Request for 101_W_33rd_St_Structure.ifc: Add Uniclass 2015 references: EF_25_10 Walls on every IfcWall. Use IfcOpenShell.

First a look at what the model holds.

```python
import ifcopenshell

model = ifcopenshell.open("101_W_33rd_St_Structure.ifc")
print(model.schema)
print("classifications:", [c.Name for c in model.by_type("IfcClassification")])
for ifc_class in ("IfcDoor", "IfcRoof", "IfcStair", "IfcWall", "IfcWindow"):
    print(ifc_class, len(model.by_type(ifc_class)))
```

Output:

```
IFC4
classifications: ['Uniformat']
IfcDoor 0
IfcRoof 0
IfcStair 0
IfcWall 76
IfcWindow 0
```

```python
import ifcopenshell
import ifcopenshell.api.classification

model = ifcopenshell.open("101_W_33rd_St_Structure.ifc")

system = ifcopenshell.api.classification.add_classification(model, classification="Uniclass 2015")

codes = {
    "IfcWall": ("EF_25_10", "Walls"),
}
for ifc_class, (code, name) in codes.items():
    products = model.by_type(ifc_class)
    ifcopenshell.api.classification.add_reference(
        model, products=products, classification=system, identification=code, name=name
    )
    print(code, len(products))

model.write("101_W_33rd_St_Structure_updated.ifc")
```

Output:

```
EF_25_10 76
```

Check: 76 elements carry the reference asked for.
